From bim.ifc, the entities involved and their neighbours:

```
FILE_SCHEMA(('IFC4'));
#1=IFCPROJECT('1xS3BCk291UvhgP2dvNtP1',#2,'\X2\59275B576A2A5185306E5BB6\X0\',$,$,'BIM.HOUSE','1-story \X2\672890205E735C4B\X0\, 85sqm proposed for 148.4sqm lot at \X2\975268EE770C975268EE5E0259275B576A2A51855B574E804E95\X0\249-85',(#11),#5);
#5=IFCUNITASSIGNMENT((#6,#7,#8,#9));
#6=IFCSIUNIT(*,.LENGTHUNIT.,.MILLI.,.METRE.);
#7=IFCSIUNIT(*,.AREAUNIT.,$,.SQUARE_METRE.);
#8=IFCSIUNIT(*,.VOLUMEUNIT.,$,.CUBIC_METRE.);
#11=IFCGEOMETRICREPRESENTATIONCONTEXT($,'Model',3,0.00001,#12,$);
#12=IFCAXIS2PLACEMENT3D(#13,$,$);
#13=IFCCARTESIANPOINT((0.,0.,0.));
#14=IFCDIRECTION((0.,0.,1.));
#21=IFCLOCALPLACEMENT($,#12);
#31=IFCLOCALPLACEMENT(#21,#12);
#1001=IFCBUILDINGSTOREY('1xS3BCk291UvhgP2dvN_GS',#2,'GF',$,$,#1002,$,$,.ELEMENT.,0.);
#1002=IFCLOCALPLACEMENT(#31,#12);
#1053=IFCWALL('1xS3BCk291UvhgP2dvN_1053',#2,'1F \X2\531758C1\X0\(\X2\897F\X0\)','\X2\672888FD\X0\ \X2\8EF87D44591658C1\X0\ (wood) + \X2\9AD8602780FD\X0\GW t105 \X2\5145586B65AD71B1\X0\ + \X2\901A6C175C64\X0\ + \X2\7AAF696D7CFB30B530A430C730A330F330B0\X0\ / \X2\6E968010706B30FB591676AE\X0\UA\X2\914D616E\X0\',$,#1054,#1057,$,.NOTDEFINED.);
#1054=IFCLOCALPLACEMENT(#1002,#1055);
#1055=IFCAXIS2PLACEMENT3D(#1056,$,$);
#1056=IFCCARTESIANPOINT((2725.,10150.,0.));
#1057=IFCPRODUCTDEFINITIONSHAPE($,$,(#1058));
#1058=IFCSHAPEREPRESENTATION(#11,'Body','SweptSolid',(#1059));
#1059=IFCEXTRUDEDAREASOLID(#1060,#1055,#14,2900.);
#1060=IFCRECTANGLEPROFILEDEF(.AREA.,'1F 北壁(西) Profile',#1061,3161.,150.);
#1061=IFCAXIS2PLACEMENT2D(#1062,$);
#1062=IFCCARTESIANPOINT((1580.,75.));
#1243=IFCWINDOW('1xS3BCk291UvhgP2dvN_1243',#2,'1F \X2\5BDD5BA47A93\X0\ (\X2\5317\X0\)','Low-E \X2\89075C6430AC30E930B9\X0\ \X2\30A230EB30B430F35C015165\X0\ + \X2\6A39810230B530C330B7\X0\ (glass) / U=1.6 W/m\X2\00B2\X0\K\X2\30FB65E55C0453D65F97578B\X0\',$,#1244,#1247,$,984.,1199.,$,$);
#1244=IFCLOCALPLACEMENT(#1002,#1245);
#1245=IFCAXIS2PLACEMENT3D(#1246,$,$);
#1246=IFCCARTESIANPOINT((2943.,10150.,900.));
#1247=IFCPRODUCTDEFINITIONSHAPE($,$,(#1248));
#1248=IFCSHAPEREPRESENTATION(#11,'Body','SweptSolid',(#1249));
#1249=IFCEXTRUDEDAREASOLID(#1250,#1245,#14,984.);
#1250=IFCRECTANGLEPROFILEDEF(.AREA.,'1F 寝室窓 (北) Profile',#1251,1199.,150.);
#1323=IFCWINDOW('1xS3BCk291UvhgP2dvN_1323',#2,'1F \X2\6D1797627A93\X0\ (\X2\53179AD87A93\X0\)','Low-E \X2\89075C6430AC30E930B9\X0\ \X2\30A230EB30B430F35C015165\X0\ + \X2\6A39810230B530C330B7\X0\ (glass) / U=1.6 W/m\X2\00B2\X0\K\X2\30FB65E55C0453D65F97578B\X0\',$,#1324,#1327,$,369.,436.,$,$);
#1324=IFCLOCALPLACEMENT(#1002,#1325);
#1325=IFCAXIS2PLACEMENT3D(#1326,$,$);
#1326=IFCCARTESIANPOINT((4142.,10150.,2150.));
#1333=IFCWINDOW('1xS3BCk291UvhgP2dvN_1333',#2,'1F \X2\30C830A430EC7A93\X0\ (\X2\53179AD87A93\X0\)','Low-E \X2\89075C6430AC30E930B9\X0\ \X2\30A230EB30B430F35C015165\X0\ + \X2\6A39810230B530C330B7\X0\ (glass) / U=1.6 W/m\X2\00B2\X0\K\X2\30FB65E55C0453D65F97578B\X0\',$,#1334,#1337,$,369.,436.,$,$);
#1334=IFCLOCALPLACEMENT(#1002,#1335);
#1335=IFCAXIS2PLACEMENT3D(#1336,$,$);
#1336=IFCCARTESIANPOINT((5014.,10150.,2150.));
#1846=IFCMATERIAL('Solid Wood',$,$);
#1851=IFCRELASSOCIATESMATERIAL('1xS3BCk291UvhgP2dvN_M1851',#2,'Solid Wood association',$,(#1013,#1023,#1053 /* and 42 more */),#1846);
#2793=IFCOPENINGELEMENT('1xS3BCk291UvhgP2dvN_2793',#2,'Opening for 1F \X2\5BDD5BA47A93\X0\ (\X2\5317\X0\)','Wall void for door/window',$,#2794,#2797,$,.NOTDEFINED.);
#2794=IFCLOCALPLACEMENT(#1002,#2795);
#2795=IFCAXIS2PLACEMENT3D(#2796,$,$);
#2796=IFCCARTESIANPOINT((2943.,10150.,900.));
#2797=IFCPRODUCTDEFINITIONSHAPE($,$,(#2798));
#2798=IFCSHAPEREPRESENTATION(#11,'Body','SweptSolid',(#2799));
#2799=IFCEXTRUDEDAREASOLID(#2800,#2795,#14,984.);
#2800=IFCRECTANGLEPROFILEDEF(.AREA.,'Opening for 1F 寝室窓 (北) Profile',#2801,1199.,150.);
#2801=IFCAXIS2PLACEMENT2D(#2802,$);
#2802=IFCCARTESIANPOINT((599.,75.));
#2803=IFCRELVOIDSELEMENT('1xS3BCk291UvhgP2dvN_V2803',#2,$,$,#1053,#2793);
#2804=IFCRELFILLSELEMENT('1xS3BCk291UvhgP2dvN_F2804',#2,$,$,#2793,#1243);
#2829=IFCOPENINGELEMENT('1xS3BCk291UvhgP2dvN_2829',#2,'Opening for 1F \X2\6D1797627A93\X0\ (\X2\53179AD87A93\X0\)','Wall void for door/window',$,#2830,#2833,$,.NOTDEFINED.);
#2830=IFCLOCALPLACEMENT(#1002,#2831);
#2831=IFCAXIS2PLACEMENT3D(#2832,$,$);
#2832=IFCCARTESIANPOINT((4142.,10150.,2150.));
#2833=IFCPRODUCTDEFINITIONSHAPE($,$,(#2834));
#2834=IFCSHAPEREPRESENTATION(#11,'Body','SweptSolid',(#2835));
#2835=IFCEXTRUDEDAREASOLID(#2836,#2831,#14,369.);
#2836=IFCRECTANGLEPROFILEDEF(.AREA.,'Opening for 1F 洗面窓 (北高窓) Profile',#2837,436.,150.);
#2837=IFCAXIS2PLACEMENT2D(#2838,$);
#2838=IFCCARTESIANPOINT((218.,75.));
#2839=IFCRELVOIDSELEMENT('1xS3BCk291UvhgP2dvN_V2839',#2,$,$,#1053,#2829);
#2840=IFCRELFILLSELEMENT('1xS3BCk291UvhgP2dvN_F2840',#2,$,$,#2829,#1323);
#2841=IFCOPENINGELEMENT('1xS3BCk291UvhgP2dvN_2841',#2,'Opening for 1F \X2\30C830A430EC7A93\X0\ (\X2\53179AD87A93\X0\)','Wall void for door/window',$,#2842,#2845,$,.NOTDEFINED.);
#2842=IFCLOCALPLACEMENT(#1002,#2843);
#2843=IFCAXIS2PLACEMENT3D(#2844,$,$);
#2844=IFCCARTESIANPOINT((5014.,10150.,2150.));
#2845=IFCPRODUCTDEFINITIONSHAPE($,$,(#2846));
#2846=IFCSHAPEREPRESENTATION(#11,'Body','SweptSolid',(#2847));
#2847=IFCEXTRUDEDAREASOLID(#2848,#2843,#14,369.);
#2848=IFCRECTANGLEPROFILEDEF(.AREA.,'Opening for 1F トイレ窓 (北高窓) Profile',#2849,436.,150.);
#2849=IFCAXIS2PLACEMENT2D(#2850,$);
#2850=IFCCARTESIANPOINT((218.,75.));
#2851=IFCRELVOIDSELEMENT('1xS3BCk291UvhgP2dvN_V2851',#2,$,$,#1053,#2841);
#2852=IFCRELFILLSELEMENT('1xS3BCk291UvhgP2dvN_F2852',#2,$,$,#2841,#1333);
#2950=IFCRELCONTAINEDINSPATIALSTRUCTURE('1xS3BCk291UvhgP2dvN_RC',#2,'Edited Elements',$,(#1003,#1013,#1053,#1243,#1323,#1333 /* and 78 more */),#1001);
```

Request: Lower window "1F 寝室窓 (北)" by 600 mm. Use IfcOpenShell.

```python
import numpy as np
import ifcopenshell
import ifcopenshell.api.geometry
import ifcopenshell.util.placement
import ifcopenshell.util.unit

model = ifcopenshell.open("bim.ifc")
unit_scale = ifcopenshell.util.unit.calculate_unit_scale(model)

window = model.by_guid("1xS3BCk291UvhgP2dvN_1243")
opening = window.FillsVoids[0].RelatingOpeningElement
dz = -600.0

shift = np.array([0.0, 0.0, dz])
# The window is not placed relative to its opening, so move both.
for product in (opening, window):
    matrix = ifcopenshell.util.placement.get_local_placement(product.ObjectPlacement)
    matrix[:3, 3] += shift
    ifcopenshell.api.geometry.edit_object_placement(model, product=product, matrix=matrix, is_si=False)

print(f"moved by {dz * unit_scale:+.3f} m")

model.write("bim_updated.ifc")
```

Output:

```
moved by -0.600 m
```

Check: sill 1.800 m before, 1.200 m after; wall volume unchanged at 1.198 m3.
